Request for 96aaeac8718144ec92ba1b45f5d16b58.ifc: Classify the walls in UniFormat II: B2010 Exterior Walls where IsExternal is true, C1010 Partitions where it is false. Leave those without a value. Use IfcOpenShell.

First a look at what the model holds.

```python
import ifcopenshell
import ifcopenshell.util.element

model = ifcopenshell.open("96aaeac8718144ec92ba1b45f5d16b58.ifc")
print(model.schema)
print("classifications:", [c.Name for c in model.by_type("IfcClassification")])
values = [ifcopenshell.util.element.get_pset(e, "Pset_WallCommon", "IsExternal") for e in model.by_type("IfcWall")]
for value in (True, False, None):
    print("IsExternal", value, values.count(value))
```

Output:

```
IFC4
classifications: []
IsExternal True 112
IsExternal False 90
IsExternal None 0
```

```python
import ifcopenshell
import ifcopenshell.api.classification
import ifcopenshell.util.element

model = ifcopenshell.open("96aaeac8718144ec92ba1b45f5d16b58.ifc")

system = ifcopenshell.api.classification.add_classification(model, classification="UniFormat II")

walls = model.by_type("IfcWall")
external = {e: ifcopenshell.util.element.get_pset(e, "Pset_WallCommon", "IsExternal") for e in walls}
for flag, code, name in ((True, "B2010", "Exterior Walls"), (False, "C1010", "Partitions")):
    products = [e for e in walls if external[e] is flag]
    ifcopenshell.api.classification.add_reference(
        model, products=products, classification=system, identification=code, name=name
    )
    print(code, len(products))

model.write("96aaeac8718144ec92ba1b45f5d16b58_updated.ifc")
```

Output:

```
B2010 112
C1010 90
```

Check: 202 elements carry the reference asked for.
